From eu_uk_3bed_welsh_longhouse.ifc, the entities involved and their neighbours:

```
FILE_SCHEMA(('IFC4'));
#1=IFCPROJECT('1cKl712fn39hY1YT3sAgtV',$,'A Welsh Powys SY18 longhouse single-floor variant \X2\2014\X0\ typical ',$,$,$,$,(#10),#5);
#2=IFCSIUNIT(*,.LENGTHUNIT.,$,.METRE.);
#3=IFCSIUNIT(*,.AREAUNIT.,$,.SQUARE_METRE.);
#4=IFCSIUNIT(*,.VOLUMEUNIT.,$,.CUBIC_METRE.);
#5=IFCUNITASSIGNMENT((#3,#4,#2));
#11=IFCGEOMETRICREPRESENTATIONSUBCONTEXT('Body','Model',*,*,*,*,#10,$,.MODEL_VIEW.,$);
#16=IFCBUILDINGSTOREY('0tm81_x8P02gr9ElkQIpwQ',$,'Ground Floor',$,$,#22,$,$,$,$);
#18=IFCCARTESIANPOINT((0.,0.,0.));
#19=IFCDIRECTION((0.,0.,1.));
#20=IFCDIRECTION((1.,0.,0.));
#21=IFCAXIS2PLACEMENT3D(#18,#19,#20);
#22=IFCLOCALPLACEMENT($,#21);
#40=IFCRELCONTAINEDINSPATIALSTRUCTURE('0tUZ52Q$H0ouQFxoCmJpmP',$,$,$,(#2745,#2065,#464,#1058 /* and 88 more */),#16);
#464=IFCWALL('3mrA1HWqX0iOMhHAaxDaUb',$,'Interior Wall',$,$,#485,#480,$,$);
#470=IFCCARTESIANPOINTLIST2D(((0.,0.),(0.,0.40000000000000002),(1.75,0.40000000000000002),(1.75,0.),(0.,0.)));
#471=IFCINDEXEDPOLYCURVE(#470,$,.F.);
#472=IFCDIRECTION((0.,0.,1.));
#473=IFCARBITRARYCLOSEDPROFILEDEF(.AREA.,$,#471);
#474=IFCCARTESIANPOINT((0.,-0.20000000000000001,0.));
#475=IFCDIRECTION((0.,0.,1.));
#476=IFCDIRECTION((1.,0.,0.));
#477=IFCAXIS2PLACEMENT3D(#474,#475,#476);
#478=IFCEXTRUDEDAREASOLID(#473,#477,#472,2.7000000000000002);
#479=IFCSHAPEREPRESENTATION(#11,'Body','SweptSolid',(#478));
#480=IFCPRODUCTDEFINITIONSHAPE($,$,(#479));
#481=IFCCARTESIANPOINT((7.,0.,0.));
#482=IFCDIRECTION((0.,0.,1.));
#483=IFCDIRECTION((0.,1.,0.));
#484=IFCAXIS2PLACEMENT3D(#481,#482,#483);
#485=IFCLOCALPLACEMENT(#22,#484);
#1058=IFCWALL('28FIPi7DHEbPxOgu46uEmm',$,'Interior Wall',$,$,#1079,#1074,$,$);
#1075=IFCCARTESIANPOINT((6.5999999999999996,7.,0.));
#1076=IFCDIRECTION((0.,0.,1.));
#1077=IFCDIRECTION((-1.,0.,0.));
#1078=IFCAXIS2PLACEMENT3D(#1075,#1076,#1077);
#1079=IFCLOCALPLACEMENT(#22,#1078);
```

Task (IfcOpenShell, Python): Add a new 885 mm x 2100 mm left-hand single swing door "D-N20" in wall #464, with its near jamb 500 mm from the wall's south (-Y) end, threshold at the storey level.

```python
import numpy as np
import ifcopenshell
import ifcopenshell.api.feature
import ifcopenshell.api.geometry
import ifcopenshell.api.root
import ifcopenshell.api.spatial
import ifcopenshell.geom
import ifcopenshell.util.element
import ifcopenshell.util.placement
import ifcopenshell.util.representation
import ifcopenshell.util.shape
import ifcopenshell.util.unit

model = ifcopenshell.open("eu_uk_3bed_welsh_longhouse.ifc")
unit_scale = ifcopenshell.util.unit.calculate_unit_scale(model)
settings = ifcopenshell.geom.settings()


def volume(element):
    """Net volume in cubic metres, openings subtracted."""
    shape = ifcopenshell.geom.create_shape(settings, element)
    return ifcopenshell.util.shape.get_volume(shape.geometry)


wall = model.by_guid("3mrA1HWqX0iOMhHAaxDaUb")
storey = ifcopenshell.util.element.get_container(wall, ifc_class="IfcBuildingStorey")
context = ifcopenshell.util.representation.get_context(model, "Model", "Body", "MODEL_VIEW")
before = volume(wall)

width, height, from_end, sill = 0.885, 2.1, 0.5, 0.0  # metres

# The wall runs along its own X axis, and the end named is its -X end.
wall_shape = ifcopenshell.geom.create_shape(settings, wall)
x, y, z = ifcopenshell.util.shape.get_vertices(wall_shape.geometry).T
start = x.min() + from_end
face, thickness = float(y.min()), float(y.max() - y.min())
wall_matrix = ifcopenshell.util.placement.get_local_placement(wall.ObjectPlacement)
level = ifcopenshell.util.placement.get_local_placement(storey.ObjectPlacement)[2, 3]


def in_wall(x, y):
    """Placement at x, y metres in the wall's axes, at sill height."""
    matrix = wall_matrix.copy()
    matrix[:, 3] = wall_matrix @ np.array([x / unit_scale, y / unit_scale, 0.0, 1.0])
    matrix[2, 3] = level + sill / unit_scale
    return matrix


# Opening: a box that overshoots both wall faces by 50 mm.
opening = ifcopenshell.api.root.create_entity(model, ifc_class="IfcOpeningElement", predefined_type="OPENING")
box = ifcopenshell.api.geometry.add_wall_representation(
    model, context=context, length=width, height=height, thickness=thickness + 0.1
)
ifcopenshell.api.geometry.assign_representation(model, product=opening, representation=box)
ifcopenshell.api.geometry.edit_object_placement(model, product=opening, matrix=in_wall(start, face - 0.05), is_si=False)
ifcopenshell.api.feature.add_feature(model, feature=opening, element=wall)

door = ifcopenshell.api.root.create_entity(model, ifc_class="IfcDoor", name="D-N20", predefined_type="DOOR")
door.OverallWidth, door.OverallHeight = width / unit_scale, height / unit_scale
door.OperationType = "SINGLE_SWING_LEFT"
body = ifcopenshell.api.geometry.add_door_representation(
    model,
    context=context,
    overall_width=door.OverallWidth,
    overall_height=door.OverallHeight,
    operation_type="SINGLE_SWING_LEFT",
    lining_properties={"LiningDepth": thickness / unit_scale, "ThresholdDepth": thickness / unit_scale},
)
ifcopenshell.api.geometry.assign_representation(model, product=door, representation=body)
ifcopenshell.api.spatial.assign_container(model, products=[door], relating_structure=storey)
ifcopenshell.api.feature.add_filling(model, opening=opening, element=door)

# The lining spans the wall, so the door starts at the wall face.
ifcopenshell.api.geometry.edit_object_placement(model, product=door, matrix=in_wall(start, face), is_si=False)

after = volume(wall)

print(f"wall volume {before:.3f} -> {after:.3f} m3")

model.write("eu_uk_3bed_welsh_longhouse_updated.ifc")
```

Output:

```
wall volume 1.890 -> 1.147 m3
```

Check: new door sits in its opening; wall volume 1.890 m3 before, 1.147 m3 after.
